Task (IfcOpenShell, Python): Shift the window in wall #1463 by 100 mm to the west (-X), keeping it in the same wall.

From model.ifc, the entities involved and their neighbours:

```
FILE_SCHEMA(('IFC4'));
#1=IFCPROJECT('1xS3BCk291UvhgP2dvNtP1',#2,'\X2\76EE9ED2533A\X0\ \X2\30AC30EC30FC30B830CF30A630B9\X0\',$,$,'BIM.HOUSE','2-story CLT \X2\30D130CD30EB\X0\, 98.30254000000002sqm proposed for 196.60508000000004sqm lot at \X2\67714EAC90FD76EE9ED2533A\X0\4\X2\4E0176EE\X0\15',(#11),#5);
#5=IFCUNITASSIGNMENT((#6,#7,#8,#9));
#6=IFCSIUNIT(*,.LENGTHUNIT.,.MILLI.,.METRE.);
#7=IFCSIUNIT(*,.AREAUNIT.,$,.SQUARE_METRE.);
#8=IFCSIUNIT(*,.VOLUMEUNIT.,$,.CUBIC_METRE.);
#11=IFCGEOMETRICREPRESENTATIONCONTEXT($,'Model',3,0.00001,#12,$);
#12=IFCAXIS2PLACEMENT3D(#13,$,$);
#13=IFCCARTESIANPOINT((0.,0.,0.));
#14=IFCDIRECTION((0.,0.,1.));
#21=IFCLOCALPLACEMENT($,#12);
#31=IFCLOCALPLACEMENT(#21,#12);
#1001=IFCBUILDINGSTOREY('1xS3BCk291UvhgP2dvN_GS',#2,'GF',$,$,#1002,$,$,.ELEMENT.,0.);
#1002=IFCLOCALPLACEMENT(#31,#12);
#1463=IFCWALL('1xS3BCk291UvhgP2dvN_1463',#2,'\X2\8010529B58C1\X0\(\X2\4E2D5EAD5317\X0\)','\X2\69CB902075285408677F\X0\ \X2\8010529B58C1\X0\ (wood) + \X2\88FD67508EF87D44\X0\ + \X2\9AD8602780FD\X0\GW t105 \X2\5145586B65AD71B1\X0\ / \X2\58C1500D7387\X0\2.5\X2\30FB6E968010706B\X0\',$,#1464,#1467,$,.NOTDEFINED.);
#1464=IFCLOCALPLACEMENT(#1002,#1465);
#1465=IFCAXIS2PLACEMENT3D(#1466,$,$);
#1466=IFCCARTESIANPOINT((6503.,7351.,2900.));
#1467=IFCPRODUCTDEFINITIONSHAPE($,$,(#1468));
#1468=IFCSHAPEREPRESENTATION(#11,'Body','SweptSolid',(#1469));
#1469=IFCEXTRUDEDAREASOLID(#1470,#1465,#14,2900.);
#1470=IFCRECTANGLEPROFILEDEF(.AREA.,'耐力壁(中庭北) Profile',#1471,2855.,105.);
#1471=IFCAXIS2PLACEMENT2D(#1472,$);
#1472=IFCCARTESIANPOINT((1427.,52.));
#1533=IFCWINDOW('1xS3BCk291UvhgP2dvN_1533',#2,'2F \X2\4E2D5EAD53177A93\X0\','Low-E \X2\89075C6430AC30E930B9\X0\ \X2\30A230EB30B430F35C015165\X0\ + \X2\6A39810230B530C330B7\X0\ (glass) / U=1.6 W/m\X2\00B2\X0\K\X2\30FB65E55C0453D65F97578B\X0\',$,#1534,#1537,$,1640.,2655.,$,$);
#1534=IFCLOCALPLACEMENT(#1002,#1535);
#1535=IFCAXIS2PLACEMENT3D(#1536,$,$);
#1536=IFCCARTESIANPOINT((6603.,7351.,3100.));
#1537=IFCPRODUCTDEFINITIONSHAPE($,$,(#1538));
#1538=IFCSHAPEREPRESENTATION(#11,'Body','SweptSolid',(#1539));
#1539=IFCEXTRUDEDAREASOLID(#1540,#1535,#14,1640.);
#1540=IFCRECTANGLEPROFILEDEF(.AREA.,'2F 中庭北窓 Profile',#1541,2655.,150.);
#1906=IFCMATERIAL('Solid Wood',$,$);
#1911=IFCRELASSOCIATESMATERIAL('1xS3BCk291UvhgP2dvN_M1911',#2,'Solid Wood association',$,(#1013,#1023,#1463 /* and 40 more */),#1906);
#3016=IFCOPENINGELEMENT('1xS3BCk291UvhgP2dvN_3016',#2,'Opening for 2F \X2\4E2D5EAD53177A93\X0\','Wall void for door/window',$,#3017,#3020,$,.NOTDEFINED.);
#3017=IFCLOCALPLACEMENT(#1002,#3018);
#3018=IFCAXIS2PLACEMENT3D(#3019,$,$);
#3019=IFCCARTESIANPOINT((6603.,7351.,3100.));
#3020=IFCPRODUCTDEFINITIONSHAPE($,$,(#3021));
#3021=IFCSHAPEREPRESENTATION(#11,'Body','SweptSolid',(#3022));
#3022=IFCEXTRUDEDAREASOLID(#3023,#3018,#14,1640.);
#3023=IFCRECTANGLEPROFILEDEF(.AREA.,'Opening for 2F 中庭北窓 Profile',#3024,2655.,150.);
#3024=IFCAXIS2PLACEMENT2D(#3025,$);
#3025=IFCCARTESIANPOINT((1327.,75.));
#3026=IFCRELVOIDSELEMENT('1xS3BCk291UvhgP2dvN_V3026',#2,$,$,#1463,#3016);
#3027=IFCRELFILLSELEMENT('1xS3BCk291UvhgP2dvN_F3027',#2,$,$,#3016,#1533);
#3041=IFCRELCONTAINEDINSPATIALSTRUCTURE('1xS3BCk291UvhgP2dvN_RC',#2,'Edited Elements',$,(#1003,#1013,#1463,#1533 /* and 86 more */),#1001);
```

```python
import ifcopenshell
import ifcopenshell.api.geometry
import ifcopenshell.util.placement
import ifcopenshell.util.unit

model = ifcopenshell.open("model.ifc")
unit_scale = ifcopenshell.util.unit.calculate_unit_scale(model)

window = model.by_guid("1xS3BCk291UvhgP2dvN_1533")
opening = window.FillsVoids[0].RelatingOpeningElement
wall = opening.VoidsElements[0].RelatingBuildingElement

wall_matrix = ifcopenshell.util.placement.get_local_placement(wall.ObjectPlacement)
shift = wall_matrix[:3, 0] * -0.1 / unit_scale
before = ifcopenshell.util.placement.get_local_placement(window.ObjectPlacement)[:3, 3].copy()

# The window is not placed relative to its opening, so move both.
for product in (opening, window):
    matrix = ifcopenshell.util.placement.get_local_placement(product.ObjectPlacement)
    matrix[:3, 3] += shift
    ifcopenshell.api.geometry.edit_object_placement(model, product=product, matrix=matrix, is_si=False)

after = ifcopenshell.util.placement.get_local_placement(window.ObjectPlacement)[:3, 3]
print("window moved by", (after - before).round(3) + 0.0)

model.write("model_rev.ifc")
```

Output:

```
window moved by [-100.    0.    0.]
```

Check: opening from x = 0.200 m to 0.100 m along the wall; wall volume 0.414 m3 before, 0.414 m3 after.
